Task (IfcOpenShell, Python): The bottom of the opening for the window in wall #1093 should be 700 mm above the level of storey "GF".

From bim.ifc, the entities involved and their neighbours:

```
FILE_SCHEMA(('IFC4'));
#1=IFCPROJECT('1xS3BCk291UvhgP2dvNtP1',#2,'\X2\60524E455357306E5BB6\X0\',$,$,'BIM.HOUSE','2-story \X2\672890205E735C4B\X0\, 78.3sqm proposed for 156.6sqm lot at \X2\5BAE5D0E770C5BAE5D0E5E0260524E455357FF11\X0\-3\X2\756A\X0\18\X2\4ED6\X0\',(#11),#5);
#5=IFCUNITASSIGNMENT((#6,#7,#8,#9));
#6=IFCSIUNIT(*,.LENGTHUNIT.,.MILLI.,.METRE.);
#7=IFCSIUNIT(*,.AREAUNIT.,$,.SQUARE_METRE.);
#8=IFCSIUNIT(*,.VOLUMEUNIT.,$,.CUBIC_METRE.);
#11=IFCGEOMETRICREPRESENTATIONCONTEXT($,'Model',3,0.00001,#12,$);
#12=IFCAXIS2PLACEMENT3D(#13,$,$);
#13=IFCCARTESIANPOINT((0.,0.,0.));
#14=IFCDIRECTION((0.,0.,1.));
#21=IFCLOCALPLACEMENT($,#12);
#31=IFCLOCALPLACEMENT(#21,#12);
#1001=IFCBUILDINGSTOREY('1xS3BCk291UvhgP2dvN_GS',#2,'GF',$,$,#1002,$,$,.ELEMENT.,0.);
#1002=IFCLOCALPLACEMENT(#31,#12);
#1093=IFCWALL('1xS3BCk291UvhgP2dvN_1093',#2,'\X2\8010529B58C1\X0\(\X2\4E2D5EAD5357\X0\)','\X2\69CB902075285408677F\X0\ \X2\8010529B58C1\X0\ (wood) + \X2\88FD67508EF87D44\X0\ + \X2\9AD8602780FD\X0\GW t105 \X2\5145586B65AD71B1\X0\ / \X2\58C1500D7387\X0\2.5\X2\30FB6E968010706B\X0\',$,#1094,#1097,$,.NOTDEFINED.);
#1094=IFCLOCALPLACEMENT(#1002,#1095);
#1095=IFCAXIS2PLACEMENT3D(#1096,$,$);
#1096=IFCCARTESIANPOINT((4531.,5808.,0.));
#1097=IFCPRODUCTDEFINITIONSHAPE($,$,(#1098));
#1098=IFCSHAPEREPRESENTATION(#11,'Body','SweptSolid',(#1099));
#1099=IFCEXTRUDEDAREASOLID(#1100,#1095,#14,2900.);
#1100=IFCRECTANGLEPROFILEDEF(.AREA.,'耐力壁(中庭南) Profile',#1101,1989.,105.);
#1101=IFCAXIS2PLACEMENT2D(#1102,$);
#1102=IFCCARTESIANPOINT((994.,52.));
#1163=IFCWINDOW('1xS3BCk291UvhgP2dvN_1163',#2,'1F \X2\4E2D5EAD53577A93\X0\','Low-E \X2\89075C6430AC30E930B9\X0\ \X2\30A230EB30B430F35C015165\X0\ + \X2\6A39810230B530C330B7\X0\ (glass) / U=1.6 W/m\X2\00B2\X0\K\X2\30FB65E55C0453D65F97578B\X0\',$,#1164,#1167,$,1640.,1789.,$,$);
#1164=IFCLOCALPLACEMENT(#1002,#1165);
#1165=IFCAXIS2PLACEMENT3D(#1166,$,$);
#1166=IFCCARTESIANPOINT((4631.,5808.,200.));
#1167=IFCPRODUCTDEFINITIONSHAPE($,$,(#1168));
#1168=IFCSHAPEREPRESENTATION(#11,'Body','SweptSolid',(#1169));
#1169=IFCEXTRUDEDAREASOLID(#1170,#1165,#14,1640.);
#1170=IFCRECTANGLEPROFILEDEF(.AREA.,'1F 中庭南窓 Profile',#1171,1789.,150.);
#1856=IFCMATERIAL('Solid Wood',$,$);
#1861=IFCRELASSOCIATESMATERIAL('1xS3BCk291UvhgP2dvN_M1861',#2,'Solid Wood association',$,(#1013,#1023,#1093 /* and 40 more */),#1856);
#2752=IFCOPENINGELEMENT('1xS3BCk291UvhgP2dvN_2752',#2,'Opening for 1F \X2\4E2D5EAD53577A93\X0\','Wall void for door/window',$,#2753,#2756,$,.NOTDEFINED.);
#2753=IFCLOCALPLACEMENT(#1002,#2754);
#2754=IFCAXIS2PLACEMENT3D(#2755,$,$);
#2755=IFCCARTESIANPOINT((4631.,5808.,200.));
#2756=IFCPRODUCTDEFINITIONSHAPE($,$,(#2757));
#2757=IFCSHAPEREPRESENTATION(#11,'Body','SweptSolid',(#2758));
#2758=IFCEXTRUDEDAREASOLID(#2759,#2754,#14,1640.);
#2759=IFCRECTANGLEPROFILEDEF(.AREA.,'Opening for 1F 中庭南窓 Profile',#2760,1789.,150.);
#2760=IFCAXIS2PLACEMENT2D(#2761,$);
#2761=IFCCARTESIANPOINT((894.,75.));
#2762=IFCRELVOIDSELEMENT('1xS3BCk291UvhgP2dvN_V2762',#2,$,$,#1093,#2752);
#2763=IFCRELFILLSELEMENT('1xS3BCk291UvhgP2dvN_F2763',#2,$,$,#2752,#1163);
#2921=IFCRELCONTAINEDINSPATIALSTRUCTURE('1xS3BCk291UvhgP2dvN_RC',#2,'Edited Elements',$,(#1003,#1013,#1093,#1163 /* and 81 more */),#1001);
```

```python
import numpy as np
import ifcopenshell
import ifcopenshell.api.geometry
import ifcopenshell.geom
import ifcopenshell.util.element
import ifcopenshell.util.placement
import ifcopenshell.util.shape
import ifcopenshell.util.unit

model = ifcopenshell.open("bim.ifc")
unit_scale = ifcopenshell.util.unit.calculate_unit_scale(model)

window = model.by_guid("1xS3BCk291UvhgP2dvN_1163")
opening = window.FillsVoids[0].RelatingOpeningElement
storey = ifcopenshell.util.element.get_container(window, ifc_class="IfcBuildingStorey")
level = ifcopenshell.util.placement.get_local_placement(storey.ObjectPlacement)[2, 3]

# The opening's origin need not be at the sill, so measure its lowest point.
shape = ifcopenshell.geom.create_shape(ifcopenshell.geom.settings(), opening)
bottom = ifcopenshell.util.shape.get_shape_bottom_elevation(shape, shape.geometry) / unit_scale
dz = level + 700.0 - bottom

shift = np.array([0.0, 0.0, dz])
# The window is not placed relative to its opening, so move both.
for product in (opening, window):
    matrix = ifcopenshell.util.placement.get_local_placement(product.ObjectPlacement)
    matrix[:3, 3] += shift
    ifcopenshell.api.geometry.edit_object_placement(model, product=product, matrix=matrix, is_si=False)

print(f"moved by {dz * unit_scale:+.3f} m")

model.write("bim_updated.ifc")
```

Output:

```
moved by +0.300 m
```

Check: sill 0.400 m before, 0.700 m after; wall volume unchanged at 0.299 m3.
